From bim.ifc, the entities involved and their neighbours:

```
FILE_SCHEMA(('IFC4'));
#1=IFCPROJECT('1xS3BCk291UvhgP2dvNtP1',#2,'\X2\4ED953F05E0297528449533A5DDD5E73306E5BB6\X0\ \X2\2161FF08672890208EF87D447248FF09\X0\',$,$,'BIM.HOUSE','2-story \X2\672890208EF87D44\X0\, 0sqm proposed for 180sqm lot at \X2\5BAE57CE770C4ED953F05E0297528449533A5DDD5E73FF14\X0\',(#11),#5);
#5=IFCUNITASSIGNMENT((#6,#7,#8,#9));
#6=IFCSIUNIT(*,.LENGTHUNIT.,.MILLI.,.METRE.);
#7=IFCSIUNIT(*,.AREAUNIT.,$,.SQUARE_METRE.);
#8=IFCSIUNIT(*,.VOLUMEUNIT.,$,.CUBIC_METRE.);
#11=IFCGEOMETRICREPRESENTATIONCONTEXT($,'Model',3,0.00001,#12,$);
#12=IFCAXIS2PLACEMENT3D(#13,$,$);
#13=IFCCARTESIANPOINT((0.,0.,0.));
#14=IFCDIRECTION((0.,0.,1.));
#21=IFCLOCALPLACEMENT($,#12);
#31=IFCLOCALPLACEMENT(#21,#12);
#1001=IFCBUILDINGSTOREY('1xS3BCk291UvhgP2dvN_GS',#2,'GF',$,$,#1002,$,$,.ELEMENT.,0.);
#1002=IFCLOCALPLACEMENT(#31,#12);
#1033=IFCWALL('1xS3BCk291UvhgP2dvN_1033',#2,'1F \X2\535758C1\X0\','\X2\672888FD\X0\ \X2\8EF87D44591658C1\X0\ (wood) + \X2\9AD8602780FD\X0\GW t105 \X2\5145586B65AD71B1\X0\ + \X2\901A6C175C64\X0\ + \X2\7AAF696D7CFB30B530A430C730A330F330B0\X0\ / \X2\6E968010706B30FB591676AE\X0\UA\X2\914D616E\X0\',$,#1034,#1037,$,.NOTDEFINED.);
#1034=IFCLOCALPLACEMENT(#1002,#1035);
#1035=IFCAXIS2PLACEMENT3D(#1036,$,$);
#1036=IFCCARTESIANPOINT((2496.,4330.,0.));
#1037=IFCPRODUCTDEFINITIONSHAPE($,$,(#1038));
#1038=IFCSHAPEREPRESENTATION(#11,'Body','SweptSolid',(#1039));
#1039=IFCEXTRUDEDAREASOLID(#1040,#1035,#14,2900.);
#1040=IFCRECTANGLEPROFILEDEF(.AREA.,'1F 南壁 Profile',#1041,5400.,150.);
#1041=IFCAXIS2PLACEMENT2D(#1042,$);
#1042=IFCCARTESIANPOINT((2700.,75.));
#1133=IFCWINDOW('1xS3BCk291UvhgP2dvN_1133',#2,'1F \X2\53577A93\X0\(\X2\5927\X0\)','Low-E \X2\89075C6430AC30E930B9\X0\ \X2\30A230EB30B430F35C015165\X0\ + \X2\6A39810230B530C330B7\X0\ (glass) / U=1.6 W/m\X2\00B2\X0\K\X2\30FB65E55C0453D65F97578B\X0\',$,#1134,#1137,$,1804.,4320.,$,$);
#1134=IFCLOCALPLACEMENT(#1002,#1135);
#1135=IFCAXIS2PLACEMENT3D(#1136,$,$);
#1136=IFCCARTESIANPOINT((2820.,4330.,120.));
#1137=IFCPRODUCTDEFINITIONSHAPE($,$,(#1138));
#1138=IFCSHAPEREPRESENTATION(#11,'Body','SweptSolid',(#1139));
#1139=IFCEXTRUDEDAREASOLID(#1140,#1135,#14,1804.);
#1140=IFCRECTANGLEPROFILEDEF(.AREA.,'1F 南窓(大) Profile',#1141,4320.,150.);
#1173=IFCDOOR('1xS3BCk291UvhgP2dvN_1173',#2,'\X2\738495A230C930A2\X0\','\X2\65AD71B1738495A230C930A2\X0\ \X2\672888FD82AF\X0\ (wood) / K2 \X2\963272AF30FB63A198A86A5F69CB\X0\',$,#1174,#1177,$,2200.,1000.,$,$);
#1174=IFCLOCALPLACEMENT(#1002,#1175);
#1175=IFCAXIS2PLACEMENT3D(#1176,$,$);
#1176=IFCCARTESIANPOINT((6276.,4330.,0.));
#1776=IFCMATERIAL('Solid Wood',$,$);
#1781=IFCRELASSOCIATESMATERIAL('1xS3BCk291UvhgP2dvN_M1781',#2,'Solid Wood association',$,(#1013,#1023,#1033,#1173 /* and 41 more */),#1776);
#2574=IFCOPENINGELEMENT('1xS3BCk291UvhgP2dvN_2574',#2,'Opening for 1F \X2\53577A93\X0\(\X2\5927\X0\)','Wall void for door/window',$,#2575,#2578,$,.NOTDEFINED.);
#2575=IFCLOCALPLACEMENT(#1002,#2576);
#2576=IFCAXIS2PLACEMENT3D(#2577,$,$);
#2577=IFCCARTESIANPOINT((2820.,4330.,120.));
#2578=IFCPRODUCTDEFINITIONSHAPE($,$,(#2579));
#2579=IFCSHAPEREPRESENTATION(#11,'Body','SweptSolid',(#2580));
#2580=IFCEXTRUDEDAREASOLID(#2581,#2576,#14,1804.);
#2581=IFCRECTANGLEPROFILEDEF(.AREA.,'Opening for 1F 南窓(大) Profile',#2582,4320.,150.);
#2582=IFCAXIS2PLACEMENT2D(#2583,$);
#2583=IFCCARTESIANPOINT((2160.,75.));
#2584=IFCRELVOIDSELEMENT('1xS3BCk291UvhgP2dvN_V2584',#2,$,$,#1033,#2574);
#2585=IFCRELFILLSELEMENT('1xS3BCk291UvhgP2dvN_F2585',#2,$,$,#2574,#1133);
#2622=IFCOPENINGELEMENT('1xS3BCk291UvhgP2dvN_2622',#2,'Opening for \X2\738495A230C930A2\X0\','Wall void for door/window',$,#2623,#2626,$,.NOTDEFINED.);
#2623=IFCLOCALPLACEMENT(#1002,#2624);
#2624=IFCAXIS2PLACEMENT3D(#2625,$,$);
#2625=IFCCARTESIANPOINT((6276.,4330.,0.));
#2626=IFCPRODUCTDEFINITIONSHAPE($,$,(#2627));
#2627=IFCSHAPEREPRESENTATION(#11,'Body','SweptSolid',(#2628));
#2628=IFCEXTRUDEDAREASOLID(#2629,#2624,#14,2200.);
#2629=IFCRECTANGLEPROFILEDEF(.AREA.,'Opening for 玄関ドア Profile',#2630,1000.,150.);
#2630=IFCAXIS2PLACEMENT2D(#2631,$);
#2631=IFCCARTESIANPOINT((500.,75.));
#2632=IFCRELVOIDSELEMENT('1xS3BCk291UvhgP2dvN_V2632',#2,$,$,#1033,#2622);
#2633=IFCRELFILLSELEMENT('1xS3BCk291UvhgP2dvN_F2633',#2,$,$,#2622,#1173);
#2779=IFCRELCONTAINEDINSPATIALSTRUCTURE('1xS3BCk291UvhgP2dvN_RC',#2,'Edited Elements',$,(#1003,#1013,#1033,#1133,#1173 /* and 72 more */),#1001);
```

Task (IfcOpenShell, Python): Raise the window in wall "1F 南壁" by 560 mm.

```python
import numpy as np
import ifcopenshell
import ifcopenshell.api.geometry
import ifcopenshell.util.placement
import ifcopenshell.util.unit

model = ifcopenshell.open("bim.ifc")
unit_scale = ifcopenshell.util.unit.calculate_unit_scale(model)

window = model.by_id(1133)
opening = window.FillsVoids[0].RelatingOpeningElement
dz = 0.56 / unit_scale

shift = np.array([0.0, 0.0, dz])
# The window is not placed relative to its opening, so move both.
for product in (opening, window):
    matrix = ifcopenshell.util.placement.get_local_placement(product.ObjectPlacement)
    matrix[:3, 3] += shift
    ifcopenshell.api.geometry.edit_object_placement(model, product=product, matrix=matrix, is_si=False)

print(f"moved by {dz * unit_scale:+.3f} m")

model.write("bim_edited.ifc")
```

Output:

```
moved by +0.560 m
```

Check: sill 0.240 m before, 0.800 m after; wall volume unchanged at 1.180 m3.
